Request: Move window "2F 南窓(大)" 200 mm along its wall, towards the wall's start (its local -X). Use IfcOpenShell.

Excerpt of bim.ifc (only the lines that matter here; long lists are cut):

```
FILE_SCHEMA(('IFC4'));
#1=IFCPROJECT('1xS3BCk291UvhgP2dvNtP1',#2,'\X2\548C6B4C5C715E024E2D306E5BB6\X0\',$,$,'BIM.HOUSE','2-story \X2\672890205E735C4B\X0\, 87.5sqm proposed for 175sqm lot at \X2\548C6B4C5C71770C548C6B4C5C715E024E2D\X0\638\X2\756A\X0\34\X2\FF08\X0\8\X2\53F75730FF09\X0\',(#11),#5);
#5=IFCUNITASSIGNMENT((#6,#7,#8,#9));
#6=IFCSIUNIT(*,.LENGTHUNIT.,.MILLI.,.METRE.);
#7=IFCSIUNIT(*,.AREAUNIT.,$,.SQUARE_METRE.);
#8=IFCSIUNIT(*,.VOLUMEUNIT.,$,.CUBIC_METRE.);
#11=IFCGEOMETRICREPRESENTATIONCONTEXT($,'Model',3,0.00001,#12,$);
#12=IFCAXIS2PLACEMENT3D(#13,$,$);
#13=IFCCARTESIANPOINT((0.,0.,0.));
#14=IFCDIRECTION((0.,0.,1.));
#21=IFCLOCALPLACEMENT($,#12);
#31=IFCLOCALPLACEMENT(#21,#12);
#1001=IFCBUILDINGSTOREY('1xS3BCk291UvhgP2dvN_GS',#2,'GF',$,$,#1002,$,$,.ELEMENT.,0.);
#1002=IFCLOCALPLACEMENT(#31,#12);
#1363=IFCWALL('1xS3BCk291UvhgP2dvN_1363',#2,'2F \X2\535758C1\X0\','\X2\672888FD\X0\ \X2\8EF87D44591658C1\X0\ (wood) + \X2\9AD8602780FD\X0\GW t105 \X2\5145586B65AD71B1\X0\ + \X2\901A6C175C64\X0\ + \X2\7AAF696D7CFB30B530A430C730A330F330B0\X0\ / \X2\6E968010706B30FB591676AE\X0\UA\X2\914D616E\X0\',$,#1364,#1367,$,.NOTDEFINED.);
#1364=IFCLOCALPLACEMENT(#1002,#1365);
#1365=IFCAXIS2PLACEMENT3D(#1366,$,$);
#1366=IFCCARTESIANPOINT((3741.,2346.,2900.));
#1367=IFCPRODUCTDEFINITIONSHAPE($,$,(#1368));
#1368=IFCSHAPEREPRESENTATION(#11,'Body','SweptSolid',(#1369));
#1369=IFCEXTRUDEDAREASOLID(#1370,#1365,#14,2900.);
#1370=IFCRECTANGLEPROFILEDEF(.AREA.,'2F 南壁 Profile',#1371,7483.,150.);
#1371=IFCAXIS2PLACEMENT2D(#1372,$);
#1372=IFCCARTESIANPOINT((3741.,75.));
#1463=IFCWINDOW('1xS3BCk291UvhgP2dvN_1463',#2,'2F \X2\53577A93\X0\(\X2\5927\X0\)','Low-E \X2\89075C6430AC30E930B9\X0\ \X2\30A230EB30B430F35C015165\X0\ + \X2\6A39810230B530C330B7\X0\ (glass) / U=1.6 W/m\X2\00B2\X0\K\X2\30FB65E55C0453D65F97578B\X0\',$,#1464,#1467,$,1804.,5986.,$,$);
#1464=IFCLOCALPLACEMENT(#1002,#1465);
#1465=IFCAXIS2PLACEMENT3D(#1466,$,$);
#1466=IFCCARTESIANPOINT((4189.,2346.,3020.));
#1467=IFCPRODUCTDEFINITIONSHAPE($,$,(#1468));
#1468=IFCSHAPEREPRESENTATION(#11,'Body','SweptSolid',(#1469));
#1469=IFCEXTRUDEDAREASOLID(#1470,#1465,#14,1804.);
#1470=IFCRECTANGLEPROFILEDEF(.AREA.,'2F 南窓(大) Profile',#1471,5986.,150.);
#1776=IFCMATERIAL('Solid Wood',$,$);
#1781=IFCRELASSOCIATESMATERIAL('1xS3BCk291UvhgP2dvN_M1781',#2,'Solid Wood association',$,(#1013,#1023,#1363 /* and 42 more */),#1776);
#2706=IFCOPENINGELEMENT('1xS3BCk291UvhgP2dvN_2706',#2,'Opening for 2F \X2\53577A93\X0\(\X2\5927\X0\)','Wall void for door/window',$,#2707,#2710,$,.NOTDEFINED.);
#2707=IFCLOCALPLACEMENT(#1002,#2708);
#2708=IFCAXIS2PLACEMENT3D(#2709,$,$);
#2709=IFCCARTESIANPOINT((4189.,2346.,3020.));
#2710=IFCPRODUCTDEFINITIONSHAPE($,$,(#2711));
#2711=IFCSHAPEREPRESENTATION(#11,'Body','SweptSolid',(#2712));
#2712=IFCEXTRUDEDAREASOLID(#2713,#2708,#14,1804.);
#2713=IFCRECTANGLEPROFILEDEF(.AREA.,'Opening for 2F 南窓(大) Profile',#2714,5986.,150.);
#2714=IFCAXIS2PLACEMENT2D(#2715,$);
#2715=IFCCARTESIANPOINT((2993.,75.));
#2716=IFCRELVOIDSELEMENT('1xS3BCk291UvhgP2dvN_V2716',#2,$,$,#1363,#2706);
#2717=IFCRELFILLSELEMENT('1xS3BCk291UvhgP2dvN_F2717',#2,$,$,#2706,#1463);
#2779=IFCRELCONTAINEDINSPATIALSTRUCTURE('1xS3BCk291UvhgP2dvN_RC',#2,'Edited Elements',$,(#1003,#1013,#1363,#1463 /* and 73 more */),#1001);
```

```python
import ifcopenshell
import ifcopenshell.api.geometry
import ifcopenshell.util.placement

model = ifcopenshell.open("bim.ifc")

window = model.by_guid("1xS3BCk291UvhgP2dvN_1463")
opening = window.FillsVoids[0].RelatingOpeningElement
wall = opening.VoidsElements[0].RelatingBuildingElement

wall_matrix = ifcopenshell.util.placement.get_local_placement(wall.ObjectPlacement)
shift = wall_matrix[:3, 0] * -200.0
before = ifcopenshell.util.placement.get_local_placement(window.ObjectPlacement)[:3, 3].copy()

# The window is not placed relative to its opening, so move both.
for product in (opening, window):
    matrix = ifcopenshell.util.placement.get_local_placement(product.ObjectPlacement)
    matrix[:3, 3] += shift
    ifcopenshell.api.geometry.edit_object_placement(model, product=product, matrix=matrix, is_si=False)

after = ifcopenshell.util.placement.get_local_placement(window.ObjectPlacement)[:3, 3]
print("window moved by", (after - before).round(3) + 0.0)

model.write("bim_v2.ifc")
```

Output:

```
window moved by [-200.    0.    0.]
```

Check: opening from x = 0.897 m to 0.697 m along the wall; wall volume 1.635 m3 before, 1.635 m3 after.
